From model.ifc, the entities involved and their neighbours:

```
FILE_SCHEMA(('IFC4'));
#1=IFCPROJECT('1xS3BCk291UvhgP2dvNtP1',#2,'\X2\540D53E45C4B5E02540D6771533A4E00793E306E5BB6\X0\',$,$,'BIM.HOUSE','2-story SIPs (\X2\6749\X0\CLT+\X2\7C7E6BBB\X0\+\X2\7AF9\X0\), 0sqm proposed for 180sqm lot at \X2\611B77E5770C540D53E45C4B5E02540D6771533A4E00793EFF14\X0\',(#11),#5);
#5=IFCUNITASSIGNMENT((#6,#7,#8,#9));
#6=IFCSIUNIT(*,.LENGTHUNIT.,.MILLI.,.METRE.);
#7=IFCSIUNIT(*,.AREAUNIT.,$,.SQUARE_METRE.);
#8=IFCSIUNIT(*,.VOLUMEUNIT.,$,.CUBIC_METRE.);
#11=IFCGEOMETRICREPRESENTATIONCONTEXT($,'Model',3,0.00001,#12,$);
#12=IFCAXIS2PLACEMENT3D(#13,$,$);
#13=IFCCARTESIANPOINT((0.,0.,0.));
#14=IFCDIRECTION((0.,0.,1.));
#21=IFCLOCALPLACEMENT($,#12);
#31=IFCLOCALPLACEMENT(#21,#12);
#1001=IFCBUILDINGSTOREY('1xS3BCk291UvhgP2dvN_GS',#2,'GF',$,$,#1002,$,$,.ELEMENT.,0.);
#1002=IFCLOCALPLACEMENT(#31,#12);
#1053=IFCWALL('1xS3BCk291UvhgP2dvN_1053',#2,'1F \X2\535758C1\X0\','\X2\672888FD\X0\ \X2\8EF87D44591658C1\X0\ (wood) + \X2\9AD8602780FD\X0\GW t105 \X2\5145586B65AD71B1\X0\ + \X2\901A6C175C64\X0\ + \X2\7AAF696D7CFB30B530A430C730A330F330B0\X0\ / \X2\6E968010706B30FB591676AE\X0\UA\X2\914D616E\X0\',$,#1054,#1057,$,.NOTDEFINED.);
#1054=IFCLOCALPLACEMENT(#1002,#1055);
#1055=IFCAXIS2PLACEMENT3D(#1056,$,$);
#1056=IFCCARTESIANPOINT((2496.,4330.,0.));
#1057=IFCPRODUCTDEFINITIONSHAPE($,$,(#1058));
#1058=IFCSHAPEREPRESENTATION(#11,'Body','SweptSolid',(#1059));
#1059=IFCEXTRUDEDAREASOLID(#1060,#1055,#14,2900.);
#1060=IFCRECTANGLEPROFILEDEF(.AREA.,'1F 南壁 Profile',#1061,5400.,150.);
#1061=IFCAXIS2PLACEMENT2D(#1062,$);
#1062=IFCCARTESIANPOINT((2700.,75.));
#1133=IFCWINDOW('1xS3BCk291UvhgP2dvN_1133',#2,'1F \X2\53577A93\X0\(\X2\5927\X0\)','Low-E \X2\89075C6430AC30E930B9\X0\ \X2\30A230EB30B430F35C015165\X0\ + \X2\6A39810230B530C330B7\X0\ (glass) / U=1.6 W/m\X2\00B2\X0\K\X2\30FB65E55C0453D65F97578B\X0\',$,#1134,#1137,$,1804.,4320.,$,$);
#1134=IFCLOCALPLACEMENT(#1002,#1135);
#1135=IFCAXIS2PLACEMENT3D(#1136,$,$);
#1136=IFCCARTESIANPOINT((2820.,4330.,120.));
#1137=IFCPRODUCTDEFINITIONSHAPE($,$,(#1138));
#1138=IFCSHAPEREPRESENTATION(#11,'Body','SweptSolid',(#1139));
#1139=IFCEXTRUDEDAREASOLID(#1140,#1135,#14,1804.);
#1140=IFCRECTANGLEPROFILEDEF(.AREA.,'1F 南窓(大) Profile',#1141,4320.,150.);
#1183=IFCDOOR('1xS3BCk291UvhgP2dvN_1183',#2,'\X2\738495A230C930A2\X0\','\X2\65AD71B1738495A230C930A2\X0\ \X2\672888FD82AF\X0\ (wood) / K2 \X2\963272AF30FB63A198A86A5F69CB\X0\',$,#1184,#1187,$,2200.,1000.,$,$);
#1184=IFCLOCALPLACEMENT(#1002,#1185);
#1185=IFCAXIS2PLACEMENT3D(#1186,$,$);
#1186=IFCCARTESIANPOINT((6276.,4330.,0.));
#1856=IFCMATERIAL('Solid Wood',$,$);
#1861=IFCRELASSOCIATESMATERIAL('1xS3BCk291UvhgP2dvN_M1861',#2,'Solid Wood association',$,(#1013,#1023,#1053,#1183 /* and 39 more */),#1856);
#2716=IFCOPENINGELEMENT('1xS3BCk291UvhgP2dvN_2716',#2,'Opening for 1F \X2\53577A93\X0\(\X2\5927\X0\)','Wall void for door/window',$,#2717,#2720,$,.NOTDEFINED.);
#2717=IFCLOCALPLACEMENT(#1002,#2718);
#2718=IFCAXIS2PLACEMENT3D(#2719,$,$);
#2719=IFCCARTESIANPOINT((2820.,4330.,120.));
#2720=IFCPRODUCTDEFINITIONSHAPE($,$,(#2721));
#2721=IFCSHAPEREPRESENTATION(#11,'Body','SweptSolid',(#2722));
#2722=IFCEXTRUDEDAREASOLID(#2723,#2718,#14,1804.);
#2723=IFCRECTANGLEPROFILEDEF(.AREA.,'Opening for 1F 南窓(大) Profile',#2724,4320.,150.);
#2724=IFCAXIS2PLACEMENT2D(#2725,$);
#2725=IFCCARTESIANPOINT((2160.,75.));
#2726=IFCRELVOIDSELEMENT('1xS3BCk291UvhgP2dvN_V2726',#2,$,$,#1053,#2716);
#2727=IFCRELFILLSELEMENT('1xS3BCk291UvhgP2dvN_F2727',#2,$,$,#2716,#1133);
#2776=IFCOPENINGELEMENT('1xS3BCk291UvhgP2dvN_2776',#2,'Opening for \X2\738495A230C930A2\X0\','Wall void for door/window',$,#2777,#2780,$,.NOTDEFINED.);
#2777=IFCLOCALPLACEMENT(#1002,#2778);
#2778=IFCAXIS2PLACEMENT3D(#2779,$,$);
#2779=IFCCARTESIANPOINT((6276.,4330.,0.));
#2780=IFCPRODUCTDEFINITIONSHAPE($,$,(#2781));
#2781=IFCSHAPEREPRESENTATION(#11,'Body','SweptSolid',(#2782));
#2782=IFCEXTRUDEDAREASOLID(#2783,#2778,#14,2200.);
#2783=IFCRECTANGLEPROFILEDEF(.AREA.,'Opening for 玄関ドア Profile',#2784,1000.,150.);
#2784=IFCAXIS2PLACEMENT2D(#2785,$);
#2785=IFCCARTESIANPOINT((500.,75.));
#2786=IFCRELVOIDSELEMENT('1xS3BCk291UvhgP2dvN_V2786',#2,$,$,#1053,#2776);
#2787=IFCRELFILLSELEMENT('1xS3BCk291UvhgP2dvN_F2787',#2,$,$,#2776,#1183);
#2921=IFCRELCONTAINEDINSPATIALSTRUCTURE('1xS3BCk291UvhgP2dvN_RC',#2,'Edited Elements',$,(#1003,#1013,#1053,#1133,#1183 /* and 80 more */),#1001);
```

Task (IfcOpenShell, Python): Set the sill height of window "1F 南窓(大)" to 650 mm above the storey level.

```python
import numpy as np
import ifcopenshell
import ifcopenshell.api.geometry
import ifcopenshell.geom
import ifcopenshell.util.element
import ifcopenshell.util.placement
import ifcopenshell.util.shape
import ifcopenshell.util.unit

model = ifcopenshell.open("model.ifc")
unit_scale = ifcopenshell.util.unit.calculate_unit_scale(model)

window = model.by_guid("1xS3BCk291UvhgP2dvN_1133")
opening = window.FillsVoids[0].RelatingOpeningElement
storey = ifcopenshell.util.element.get_container(window, ifc_class="IfcBuildingStorey")
level = ifcopenshell.util.placement.get_local_placement(storey.ObjectPlacement)[2, 3]

# The opening's origin need not be at the sill, so measure its lowest point.
shape = ifcopenshell.geom.create_shape(ifcopenshell.geom.settings(), opening)
bottom = ifcopenshell.util.shape.get_shape_bottom_elevation(shape, shape.geometry) / unit_scale
dz = level + 650.0 - bottom

shift = np.array([0.0, 0.0, dz])
# The window is not placed relative to its opening, so move both.
for product in (opening, window):
    matrix = ifcopenshell.util.placement.get_local_placement(product.ObjectPlacement)
    matrix[:3, 3] += shift
    ifcopenshell.api.geometry.edit_object_placement(model, product=product, matrix=matrix, is_si=False)

print(f"moved by {dz * unit_scale:+.3f} m")

model.write("model_v2.ifc")
```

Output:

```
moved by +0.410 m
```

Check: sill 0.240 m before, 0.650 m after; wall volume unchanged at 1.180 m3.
